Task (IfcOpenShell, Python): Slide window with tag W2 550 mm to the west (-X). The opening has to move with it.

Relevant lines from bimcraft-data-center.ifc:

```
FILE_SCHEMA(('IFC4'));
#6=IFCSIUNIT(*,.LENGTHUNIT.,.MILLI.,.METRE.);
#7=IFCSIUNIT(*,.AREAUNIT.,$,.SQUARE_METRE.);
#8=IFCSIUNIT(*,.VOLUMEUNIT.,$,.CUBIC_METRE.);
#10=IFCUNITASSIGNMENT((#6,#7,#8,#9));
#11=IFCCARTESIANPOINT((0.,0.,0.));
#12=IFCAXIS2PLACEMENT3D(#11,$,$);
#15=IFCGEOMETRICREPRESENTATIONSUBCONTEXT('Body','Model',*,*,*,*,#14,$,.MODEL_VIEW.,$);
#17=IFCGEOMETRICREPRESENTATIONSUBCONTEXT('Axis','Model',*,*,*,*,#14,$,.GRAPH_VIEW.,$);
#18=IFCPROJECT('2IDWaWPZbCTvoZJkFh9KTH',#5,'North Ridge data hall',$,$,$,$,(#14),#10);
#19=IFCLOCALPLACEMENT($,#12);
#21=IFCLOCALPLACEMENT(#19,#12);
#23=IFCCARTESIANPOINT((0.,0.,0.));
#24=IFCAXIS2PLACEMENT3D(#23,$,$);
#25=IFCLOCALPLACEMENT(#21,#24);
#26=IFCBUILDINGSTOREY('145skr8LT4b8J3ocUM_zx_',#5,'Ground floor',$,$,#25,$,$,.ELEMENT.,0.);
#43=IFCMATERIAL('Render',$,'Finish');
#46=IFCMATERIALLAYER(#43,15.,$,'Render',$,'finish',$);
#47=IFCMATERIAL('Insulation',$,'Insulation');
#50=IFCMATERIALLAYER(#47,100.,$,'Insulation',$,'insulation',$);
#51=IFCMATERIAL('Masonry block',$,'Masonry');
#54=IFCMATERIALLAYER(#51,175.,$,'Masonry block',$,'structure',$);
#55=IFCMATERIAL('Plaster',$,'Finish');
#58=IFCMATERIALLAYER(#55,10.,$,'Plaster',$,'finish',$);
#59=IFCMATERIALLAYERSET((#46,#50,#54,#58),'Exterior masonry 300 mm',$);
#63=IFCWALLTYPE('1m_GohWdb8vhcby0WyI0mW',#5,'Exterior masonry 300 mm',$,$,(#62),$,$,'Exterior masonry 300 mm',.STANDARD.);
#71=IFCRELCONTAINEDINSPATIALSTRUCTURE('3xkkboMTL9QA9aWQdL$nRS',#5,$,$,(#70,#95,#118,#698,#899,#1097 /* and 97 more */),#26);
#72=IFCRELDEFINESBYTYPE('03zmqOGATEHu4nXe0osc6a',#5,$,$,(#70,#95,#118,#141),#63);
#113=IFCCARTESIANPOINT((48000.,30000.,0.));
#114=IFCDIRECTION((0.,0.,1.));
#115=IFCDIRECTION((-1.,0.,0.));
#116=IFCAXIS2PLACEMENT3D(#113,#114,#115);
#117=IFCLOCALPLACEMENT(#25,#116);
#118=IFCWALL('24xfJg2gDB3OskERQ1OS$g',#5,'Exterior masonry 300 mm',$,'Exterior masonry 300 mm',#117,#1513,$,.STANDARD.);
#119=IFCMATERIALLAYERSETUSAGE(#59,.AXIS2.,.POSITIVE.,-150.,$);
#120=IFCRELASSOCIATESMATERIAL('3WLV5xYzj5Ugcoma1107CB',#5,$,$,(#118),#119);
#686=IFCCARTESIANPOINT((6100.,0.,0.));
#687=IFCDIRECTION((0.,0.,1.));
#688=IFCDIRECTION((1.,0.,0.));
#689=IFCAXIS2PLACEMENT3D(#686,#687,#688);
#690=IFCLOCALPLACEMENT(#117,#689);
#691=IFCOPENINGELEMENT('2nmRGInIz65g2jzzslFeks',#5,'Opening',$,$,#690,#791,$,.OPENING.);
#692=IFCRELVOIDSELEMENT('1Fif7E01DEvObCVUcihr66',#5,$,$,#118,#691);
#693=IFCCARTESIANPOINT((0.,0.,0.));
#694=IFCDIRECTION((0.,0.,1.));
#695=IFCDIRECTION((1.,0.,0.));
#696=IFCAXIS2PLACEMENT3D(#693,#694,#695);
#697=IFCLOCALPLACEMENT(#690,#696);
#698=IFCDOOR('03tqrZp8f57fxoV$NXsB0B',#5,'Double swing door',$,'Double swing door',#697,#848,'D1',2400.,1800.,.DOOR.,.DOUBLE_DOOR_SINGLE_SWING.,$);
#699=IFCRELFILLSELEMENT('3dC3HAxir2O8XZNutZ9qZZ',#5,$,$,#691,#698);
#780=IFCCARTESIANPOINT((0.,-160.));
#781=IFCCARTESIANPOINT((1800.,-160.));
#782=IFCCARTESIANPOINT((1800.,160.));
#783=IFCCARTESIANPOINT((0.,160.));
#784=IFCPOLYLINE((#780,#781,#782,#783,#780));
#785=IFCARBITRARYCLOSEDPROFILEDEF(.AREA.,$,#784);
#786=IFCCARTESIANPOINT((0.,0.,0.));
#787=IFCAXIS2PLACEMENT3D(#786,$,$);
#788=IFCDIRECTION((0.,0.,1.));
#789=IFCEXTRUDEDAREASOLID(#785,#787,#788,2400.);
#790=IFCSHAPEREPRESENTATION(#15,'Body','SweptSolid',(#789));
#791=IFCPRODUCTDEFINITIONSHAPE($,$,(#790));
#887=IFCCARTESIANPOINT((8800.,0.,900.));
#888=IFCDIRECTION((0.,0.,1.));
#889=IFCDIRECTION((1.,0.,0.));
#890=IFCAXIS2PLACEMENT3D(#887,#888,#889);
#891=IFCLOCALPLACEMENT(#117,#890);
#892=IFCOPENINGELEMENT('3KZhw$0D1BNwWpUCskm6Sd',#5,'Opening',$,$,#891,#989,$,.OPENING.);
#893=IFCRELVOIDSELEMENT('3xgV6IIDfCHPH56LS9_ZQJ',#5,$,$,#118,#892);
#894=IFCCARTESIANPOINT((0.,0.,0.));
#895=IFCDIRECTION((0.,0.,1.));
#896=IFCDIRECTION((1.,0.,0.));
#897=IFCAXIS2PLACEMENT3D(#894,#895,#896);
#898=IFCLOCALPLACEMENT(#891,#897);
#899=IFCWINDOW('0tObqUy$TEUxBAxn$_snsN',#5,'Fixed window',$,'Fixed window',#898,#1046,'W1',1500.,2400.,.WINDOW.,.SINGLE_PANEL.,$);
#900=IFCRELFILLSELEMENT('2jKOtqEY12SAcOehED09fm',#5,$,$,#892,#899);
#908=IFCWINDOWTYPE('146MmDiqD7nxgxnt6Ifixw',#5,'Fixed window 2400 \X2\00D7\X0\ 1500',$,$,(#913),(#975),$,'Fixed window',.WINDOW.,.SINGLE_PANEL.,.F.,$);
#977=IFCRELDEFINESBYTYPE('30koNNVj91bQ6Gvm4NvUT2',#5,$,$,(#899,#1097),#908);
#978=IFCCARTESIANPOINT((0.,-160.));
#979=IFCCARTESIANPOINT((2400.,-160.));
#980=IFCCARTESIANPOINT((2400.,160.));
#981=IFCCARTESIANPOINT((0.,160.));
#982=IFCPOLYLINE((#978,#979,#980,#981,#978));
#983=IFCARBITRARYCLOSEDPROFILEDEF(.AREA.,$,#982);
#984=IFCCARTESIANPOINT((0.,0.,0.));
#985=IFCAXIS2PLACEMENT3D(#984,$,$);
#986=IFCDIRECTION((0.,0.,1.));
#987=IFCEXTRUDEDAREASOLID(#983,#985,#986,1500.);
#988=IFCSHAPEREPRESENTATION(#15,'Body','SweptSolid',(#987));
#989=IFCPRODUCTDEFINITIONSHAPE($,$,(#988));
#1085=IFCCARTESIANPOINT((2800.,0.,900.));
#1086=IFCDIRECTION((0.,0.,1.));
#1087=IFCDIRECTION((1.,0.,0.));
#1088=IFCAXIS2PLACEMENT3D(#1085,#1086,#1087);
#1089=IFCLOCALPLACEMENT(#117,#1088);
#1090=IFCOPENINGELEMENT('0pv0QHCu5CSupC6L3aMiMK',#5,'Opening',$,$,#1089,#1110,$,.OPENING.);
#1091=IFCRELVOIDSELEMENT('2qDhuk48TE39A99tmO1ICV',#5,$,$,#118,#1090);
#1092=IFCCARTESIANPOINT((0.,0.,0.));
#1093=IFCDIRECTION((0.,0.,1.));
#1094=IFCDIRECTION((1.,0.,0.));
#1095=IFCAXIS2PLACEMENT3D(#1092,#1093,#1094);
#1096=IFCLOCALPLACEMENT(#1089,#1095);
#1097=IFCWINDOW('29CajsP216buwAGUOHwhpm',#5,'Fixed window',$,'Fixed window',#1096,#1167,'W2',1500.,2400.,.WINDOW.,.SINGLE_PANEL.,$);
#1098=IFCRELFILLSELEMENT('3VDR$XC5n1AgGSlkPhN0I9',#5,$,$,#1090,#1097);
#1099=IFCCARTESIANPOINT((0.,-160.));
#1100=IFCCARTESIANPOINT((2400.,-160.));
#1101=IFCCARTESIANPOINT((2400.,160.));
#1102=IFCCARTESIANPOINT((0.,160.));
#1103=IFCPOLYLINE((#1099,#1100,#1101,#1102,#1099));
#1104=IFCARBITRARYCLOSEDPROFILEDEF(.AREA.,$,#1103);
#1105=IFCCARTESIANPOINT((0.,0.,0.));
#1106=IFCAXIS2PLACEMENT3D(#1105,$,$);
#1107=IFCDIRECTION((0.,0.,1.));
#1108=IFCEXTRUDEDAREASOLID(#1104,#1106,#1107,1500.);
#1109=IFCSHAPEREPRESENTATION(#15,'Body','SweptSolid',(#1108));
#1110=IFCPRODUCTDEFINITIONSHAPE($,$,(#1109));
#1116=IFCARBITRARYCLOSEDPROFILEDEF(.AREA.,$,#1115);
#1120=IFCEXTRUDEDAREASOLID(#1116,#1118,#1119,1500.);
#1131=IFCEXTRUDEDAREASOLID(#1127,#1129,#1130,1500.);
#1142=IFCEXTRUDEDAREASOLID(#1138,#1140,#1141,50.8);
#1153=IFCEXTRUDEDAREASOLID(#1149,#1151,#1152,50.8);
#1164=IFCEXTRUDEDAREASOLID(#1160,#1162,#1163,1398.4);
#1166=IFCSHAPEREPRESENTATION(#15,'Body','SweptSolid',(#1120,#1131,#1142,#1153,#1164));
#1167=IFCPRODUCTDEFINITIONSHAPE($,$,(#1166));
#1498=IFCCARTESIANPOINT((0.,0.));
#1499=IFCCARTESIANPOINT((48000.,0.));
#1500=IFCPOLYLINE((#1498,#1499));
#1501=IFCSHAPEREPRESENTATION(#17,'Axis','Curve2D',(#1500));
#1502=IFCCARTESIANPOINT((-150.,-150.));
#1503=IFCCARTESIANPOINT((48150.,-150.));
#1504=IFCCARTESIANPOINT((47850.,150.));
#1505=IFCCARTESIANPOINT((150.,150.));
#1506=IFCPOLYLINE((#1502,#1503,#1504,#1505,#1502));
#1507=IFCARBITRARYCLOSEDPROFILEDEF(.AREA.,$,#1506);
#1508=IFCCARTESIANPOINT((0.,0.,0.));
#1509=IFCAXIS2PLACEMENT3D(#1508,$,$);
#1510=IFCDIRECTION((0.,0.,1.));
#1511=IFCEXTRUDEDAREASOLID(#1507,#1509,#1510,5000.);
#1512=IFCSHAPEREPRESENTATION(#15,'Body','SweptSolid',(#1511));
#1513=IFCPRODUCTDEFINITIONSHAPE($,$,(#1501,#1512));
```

```python
import ifcopenshell
import ifcopenshell.api.geometry
import ifcopenshell.util.placement

model = ifcopenshell.open("bimcraft-data-center.ifc")

window = model.by_guid("29CajsP216buwAGUOHwhpm")
opening = window.FillsVoids[0].RelatingOpeningElement
wall = opening.VoidsElements[0].RelatingBuildingElement

wall_matrix = ifcopenshell.util.placement.get_local_placement(wall.ObjectPlacement)
shift = wall_matrix[:3, 0] * 550.0
before = ifcopenshell.util.placement.get_local_placement(window.ObjectPlacement)[:3, 3].copy()

# The window is placed relative to its opening, so it follows when the opening moves.
matrix = ifcopenshell.util.placement.get_local_placement(opening.ObjectPlacement)
matrix[:3, 3] += shift
ifcopenshell.api.geometry.edit_object_placement(
    model, product=opening, matrix=matrix, is_si=False, should_transform_children=True
)

after = ifcopenshell.util.placement.get_local_placement(window.ObjectPlacement)[:3, 3]
print("window moved by", (after - before).round(3) + 0.0)

model.write("bimcraft-data-center-out.ifc")
```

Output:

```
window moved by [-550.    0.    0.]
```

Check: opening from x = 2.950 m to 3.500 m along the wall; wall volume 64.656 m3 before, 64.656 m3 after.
